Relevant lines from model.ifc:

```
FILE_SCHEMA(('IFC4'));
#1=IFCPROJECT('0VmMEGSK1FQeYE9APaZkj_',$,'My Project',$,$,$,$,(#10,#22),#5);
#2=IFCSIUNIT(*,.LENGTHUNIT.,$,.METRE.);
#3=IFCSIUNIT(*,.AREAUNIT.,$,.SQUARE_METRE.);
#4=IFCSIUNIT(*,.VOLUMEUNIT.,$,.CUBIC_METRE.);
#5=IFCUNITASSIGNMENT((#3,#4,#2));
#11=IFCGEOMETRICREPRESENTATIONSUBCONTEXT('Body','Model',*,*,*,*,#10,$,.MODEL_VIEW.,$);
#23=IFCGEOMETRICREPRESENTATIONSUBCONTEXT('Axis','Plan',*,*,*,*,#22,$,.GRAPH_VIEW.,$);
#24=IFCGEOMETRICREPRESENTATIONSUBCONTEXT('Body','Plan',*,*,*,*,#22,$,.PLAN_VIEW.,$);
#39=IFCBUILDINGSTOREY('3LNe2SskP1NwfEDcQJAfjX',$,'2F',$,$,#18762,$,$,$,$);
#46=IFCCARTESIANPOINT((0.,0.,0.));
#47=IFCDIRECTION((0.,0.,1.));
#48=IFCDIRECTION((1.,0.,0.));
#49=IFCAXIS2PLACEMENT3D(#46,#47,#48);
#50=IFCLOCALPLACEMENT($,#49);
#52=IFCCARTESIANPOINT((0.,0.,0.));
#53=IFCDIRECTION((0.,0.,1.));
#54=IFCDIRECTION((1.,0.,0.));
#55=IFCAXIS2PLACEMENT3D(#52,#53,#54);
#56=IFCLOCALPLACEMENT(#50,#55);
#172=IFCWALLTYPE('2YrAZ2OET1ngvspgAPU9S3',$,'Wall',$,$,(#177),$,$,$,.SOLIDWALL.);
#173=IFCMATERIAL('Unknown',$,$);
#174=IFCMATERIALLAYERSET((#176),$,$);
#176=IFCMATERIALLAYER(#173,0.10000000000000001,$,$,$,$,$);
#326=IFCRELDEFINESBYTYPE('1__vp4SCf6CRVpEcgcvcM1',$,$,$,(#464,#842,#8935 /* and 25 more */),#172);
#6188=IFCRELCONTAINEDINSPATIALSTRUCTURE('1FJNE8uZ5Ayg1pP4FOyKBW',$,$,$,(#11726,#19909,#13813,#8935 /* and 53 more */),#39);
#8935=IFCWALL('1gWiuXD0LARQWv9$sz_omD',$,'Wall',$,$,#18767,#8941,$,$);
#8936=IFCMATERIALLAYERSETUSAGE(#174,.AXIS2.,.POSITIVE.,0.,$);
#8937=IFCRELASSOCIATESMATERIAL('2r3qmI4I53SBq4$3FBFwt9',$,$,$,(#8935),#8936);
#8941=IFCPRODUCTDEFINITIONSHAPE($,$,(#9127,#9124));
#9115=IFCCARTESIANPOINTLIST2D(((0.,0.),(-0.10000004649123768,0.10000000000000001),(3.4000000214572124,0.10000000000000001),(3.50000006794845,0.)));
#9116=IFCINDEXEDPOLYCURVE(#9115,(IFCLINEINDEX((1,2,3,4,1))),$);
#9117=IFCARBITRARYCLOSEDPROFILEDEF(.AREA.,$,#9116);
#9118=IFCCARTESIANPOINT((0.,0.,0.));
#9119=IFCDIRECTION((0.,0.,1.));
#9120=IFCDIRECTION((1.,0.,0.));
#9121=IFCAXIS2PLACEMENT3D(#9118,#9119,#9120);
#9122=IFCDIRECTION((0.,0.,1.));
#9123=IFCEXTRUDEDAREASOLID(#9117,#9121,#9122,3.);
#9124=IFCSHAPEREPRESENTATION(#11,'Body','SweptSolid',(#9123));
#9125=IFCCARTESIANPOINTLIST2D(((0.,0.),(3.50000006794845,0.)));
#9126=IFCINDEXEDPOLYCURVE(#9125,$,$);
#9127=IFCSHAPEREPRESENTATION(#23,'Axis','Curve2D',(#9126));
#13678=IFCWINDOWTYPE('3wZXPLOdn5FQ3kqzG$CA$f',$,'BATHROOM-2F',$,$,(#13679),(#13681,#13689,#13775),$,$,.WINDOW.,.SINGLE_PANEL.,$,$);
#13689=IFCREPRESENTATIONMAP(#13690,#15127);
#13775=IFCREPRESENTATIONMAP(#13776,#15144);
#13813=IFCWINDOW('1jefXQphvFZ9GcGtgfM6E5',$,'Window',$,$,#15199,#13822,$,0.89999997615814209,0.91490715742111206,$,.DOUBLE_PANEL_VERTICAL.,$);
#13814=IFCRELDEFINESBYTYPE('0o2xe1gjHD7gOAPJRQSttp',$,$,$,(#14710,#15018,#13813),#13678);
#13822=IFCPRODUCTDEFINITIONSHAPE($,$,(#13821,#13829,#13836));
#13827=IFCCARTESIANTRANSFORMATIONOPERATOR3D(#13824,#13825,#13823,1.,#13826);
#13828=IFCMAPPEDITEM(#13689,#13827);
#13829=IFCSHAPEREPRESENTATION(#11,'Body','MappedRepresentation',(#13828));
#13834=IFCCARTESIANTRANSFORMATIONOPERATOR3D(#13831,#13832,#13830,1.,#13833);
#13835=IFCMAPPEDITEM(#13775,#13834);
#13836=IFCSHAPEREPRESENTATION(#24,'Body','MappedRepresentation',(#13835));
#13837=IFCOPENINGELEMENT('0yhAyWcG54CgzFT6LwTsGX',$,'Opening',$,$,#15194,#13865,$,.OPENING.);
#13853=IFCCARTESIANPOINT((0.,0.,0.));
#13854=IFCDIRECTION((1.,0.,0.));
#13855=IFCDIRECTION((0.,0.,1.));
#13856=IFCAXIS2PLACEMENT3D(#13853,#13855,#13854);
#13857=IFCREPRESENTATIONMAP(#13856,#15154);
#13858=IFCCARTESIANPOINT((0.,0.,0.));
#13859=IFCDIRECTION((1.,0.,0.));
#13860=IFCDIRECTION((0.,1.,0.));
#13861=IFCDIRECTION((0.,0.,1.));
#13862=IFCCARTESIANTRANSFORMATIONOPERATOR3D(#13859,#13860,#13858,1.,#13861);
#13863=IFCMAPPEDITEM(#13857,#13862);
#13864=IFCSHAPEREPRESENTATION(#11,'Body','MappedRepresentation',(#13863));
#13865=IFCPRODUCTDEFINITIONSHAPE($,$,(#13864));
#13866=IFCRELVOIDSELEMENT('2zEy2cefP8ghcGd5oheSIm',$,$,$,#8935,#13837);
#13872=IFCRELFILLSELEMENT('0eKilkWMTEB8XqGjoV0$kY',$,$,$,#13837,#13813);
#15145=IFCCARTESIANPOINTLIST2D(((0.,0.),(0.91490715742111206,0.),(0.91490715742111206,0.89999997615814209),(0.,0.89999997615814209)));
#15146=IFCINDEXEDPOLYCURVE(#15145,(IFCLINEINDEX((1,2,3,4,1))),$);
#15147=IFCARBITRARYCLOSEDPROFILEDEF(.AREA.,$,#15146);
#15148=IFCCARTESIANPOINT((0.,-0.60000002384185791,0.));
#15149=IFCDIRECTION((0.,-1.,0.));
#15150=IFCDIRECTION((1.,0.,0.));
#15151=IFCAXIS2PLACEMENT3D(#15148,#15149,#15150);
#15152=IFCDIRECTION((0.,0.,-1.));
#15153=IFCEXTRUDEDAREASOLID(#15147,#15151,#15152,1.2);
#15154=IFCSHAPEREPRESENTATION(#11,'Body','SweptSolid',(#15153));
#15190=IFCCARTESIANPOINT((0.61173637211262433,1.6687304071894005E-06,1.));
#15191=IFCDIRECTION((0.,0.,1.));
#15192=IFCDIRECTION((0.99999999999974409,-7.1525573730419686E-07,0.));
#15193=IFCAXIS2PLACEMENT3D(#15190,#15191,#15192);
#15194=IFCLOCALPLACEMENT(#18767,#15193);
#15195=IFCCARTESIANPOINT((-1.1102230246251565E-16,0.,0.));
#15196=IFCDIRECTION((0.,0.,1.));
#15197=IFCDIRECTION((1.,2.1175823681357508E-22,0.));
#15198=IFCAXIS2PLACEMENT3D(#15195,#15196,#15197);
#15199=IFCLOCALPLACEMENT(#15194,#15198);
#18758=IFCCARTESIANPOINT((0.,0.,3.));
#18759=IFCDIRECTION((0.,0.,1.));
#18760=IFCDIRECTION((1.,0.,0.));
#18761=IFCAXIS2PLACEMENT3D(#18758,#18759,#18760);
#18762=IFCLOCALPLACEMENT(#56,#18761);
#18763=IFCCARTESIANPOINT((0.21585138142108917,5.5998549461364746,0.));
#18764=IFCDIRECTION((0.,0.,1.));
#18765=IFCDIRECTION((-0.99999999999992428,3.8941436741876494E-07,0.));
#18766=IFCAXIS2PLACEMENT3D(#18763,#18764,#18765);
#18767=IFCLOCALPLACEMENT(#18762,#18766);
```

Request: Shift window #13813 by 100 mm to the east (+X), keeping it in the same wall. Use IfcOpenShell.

```python
import ifcopenshell
import ifcopenshell.api.geometry
import ifcopenshell.util.placement
import ifcopenshell.util.unit

model = ifcopenshell.open("model.ifc")
unit_scale = ifcopenshell.util.unit.calculate_unit_scale(model)

window = model.by_guid("1jefXQphvFZ9GcGtgfM6E5")
opening = window.FillsVoids[0].RelatingOpeningElement
wall = opening.VoidsElements[0].RelatingBuildingElement

wall_matrix = ifcopenshell.util.placement.get_local_placement(wall.ObjectPlacement)
shift = wall_matrix[:3, 0] * -0.1 / unit_scale
before = ifcopenshell.util.placement.get_local_placement(window.ObjectPlacement)[:3, 3].copy()

# The window is placed relative to its opening, so it follows when the opening moves.
matrix = ifcopenshell.util.placement.get_local_placement(opening.ObjectPlacement)
matrix[:3, 3] += shift
ifcopenshell.api.geometry.edit_object_placement(
    model, product=opening, matrix=matrix, is_si=False, should_transform_children=True
)

after = ifcopenshell.util.placement.get_local_placement(window.ObjectPlacement)[:3, 3]
print("window moved by", (after - before).round(3) + 0.0)

model.write("model_updated.ifc")
```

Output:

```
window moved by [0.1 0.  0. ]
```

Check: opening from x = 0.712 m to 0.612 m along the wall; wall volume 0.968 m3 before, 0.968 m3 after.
